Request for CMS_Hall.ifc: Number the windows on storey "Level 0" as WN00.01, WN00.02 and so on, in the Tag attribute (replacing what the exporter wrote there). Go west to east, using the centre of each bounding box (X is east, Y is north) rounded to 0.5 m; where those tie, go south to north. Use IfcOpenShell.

First a look at what the model holds.

```python
import ifcopenshell
import ifcopenshell.util.element
import ifcopenshell.util.placement

model = ifcopenshell.open("CMS_Hall.ifc")
print(model.schema)
storey = next(s for s in model.by_type("IfcBuildingStorey") if s.Name == "Level 0")
windows = [e for e in ifcopenshell.util.element.get_decomposition(storey) if e.is_a("IfcWindow")]
for e in sorted(windows, key=lambda e: e.id()):
    origin = ifcopenshell.util.placement.get_local_placement(e.ObjectPlacement)[:3, 3]
    print(e.id(), e.Tag, e.Name, origin.round(2) + 0.0, sep=" | ")
```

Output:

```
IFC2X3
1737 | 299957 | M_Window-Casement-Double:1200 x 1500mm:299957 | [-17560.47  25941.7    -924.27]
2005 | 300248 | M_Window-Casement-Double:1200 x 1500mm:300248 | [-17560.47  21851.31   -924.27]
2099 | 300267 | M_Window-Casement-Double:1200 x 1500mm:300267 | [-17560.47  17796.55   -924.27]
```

```python
import ifcopenshell
import ifcopenshell.geom
import ifcopenshell.util.element
import ifcopenshell.util.shape

model = ifcopenshell.open("CMS_Hall.ifc")
settings = ifcopenshell.geom.settings()
settings.set("use-world-coords", True)


def centre(element):
    shape = ifcopenshell.geom.create_shape(settings, element)
    return ifcopenshell.util.shape.get_bbox_centroid(shape.geometry)


storey = next(s for s in model.by_type("IfcBuildingStorey") if s.Name == "Level 0")
windows = [e for e in ifcopenshell.util.element.get_decomposition(storey) if e.is_a("IfcWindow")]

# Insertion points can sit at a corner or the storey origin, so sort by the geometry (in metres).
centres = {e: centre(e) for e in windows}
windows.sort(key=lambda e: (round(centres[e][0] / 0.5), centres[e][1]))

for i, e in enumerate(windows, start=1):
    number = f"WN00.{i:02d}"
    e.Tag = number
    print(e.id(), number)

model.write("CMS_Hall_rev.ifc")
```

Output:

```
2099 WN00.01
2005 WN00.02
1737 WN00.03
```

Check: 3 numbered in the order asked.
